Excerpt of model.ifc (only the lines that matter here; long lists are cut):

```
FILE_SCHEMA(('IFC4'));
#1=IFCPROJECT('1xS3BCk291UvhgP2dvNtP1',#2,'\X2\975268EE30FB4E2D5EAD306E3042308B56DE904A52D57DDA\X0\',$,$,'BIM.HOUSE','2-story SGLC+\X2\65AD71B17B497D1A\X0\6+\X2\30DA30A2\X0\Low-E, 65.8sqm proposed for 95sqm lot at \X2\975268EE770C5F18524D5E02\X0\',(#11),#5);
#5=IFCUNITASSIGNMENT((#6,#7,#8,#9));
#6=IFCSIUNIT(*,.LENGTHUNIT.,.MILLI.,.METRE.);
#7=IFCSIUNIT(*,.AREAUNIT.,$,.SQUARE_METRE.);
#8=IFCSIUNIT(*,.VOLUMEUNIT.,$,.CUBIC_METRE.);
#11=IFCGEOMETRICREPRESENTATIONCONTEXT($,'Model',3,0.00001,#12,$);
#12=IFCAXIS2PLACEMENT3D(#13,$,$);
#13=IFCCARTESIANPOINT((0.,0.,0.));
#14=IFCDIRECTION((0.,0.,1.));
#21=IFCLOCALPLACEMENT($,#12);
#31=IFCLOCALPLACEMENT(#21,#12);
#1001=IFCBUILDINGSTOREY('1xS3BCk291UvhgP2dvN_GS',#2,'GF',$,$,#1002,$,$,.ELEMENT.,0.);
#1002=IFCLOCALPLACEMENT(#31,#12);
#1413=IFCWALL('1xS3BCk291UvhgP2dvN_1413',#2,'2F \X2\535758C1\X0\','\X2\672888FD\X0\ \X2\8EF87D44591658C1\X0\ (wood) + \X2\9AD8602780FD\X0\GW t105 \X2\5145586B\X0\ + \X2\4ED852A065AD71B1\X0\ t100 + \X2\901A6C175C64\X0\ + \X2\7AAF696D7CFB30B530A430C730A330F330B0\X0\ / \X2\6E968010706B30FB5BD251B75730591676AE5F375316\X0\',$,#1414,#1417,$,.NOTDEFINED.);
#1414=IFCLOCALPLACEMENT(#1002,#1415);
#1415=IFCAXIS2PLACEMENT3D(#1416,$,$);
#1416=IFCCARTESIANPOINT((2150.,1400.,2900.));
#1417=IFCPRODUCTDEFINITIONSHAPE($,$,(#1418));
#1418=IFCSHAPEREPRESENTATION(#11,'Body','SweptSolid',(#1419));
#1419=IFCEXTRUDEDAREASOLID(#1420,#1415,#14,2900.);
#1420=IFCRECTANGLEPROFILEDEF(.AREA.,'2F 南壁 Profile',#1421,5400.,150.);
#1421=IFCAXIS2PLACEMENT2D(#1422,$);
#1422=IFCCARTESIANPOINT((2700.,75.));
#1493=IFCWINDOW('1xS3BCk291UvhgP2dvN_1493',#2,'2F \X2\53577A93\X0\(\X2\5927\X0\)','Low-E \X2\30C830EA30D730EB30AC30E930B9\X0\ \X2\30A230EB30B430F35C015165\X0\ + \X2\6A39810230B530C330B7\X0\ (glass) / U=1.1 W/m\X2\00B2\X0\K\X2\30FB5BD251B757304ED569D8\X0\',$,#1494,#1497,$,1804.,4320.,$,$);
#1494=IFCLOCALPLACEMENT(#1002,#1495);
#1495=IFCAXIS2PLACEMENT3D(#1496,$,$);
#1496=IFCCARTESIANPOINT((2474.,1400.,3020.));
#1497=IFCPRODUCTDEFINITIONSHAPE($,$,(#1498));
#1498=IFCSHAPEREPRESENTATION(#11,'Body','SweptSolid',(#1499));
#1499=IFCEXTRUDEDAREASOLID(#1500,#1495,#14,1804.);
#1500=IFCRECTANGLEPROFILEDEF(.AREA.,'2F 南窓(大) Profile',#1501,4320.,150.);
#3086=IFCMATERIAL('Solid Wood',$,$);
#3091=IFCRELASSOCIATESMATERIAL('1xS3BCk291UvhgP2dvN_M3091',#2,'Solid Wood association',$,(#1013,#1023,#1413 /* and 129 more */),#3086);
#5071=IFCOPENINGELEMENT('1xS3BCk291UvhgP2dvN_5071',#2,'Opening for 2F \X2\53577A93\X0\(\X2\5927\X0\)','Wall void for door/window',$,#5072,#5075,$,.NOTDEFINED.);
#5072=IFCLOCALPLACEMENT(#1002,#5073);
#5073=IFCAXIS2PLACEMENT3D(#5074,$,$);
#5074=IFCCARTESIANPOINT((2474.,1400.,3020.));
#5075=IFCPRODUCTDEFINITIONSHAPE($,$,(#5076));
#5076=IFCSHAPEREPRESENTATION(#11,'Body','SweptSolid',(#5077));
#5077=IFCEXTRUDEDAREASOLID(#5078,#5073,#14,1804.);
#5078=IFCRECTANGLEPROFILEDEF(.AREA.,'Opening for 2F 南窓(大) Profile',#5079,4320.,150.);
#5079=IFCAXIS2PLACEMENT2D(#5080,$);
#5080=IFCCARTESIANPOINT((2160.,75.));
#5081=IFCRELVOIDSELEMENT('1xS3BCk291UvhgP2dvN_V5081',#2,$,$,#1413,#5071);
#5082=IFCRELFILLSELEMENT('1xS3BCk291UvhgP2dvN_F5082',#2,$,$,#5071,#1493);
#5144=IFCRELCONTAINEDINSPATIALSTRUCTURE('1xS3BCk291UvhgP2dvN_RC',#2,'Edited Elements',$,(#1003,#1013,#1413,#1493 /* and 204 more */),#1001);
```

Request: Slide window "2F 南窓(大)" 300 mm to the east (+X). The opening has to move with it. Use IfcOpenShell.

```python
import ifcopenshell
import ifcopenshell.api.geometry
import ifcopenshell.util.placement

model = ifcopenshell.open("model.ifc")

window = model.by_id(1493)
opening = window.FillsVoids[0].RelatingOpeningElement
wall = opening.VoidsElements[0].RelatingBuildingElement

wall_matrix = ifcopenshell.util.placement.get_local_placement(wall.ObjectPlacement)
shift = wall_matrix[:3, 0] * 300.0
before = ifcopenshell.util.placement.get_local_placement(window.ObjectPlacement)[:3, 3].copy()

# The window is not placed relative to its opening, so move both.
for product in (opening, window):
    matrix = ifcopenshell.util.placement.get_local_placement(product.ObjectPlacement)
    matrix[:3, 3] += shift
    ifcopenshell.api.geometry.edit_object_placement(model, product=product, matrix=matrix, is_si=False)

after = ifcopenshell.util.placement.get_local_placement(window.ObjectPlacement)[:3, 3]
print("window moved by", (after - before).round(3) + 0.0)

model.write("model_v2.ifc")
```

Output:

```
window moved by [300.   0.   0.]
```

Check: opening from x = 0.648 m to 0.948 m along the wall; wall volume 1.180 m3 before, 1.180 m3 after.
